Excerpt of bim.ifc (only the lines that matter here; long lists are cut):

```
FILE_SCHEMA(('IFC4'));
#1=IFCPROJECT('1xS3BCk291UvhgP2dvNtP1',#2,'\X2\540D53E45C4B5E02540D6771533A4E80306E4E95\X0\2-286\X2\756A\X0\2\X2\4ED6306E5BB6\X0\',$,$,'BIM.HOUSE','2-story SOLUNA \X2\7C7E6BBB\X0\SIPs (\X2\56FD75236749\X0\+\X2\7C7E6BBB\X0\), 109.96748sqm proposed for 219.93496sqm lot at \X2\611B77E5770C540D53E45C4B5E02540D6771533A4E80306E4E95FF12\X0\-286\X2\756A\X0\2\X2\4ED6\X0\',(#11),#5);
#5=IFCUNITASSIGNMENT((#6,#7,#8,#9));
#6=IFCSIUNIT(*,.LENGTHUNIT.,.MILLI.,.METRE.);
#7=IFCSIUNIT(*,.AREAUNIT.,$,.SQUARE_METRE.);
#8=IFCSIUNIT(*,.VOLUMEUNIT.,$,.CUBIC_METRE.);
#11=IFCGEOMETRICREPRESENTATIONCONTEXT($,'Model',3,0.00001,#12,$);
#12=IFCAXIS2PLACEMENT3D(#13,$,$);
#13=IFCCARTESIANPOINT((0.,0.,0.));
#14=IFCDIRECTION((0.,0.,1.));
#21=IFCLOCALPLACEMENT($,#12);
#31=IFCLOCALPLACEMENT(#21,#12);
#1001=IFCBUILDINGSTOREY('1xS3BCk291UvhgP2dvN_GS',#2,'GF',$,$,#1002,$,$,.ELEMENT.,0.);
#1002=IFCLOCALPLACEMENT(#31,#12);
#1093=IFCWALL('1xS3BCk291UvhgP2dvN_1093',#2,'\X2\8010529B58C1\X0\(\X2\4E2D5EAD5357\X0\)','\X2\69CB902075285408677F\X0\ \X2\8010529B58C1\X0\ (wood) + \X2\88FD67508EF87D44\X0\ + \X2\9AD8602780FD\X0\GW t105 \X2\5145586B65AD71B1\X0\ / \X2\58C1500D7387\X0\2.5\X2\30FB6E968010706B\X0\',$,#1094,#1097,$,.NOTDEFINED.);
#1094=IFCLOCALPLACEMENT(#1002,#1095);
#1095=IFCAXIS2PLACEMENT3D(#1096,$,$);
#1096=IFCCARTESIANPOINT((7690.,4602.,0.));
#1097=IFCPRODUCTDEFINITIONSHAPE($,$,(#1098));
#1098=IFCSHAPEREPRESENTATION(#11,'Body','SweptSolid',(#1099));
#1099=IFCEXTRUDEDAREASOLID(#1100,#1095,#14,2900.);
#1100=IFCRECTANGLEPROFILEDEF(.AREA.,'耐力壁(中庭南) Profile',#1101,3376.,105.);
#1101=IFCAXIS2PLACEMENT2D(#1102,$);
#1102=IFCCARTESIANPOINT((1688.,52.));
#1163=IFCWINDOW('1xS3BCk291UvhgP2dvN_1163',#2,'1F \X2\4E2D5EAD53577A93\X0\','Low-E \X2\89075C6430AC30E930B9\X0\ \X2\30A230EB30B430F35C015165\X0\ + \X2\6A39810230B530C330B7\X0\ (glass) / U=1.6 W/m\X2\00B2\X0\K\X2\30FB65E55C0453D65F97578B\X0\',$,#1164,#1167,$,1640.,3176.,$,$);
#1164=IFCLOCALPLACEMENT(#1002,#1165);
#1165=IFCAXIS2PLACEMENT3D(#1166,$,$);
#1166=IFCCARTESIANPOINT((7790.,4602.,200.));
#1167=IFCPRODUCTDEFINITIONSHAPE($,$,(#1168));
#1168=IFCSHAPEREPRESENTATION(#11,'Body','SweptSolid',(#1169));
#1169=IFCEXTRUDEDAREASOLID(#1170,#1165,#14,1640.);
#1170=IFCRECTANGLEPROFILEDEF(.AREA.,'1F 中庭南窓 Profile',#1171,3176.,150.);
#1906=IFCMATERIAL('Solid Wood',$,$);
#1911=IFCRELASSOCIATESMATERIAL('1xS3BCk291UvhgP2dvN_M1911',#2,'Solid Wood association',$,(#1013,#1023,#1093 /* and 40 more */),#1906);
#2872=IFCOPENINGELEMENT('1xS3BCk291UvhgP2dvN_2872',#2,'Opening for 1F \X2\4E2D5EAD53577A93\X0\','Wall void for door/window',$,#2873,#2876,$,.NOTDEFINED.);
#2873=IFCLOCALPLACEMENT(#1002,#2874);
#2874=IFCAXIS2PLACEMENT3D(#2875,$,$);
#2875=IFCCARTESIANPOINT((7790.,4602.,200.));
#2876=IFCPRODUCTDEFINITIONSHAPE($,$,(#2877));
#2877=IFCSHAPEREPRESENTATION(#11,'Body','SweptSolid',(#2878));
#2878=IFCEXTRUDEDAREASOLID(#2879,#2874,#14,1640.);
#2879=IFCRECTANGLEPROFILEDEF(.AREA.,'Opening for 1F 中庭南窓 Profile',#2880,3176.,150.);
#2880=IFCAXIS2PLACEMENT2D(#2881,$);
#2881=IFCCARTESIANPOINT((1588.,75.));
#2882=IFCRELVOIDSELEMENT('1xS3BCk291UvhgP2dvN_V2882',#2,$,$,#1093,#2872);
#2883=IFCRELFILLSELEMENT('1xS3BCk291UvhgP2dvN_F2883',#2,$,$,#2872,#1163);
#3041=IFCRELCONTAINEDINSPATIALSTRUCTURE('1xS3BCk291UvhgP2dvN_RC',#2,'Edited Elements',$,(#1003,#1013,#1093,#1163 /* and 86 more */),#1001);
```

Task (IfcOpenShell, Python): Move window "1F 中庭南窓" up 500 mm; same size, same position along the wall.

```python
import numpy as np
import ifcopenshell
import ifcopenshell.api.geometry
import ifcopenshell.util.placement
import ifcopenshell.util.unit

model = ifcopenshell.open("bim.ifc")
unit_scale = ifcopenshell.util.unit.calculate_unit_scale(model)

window = model.by_id(1163)
opening = window.FillsVoids[0].RelatingOpeningElement
dz = 0.5 / unit_scale

shift = np.array([0.0, 0.0, dz])
# The window is not placed relative to its opening, so move both.
for product in (opening, window):
    matrix = ifcopenshell.util.placement.get_local_placement(product.ObjectPlacement)
    matrix[:3, 3] += shift
    ifcopenshell.api.geometry.edit_object_placement(model, product=product, matrix=matrix, is_si=False)

print(f"moved by {dz * unit_scale:+.3f} m")

model.write("bim_rev.ifc")
```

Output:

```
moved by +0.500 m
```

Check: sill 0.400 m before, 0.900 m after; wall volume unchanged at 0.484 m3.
